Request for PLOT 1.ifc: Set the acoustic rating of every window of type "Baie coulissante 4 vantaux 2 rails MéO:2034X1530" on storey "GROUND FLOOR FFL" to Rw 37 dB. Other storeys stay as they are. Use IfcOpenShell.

First a look at what the model holds.

```python
import ifcopenshell
import ifcopenshell.util.element

model = ifcopenshell.open("PLOT 1.ifc")
print(model.schema)
storey = next(s for s in model.by_type("IfcBuildingStorey") if s.Name == "GROUND FLOOR FFL")
windows = [e for e in ifcopenshell.util.element.get_decomposition(storey) if e.is_a("IfcWindow")]
seen = {}
for e in windows:
    element_type = ifcopenshell.util.element.get_type(e)
    key = (element_type.Name if element_type != e and element_type else None, ifcopenshell.util.element.get_pset(e, "Pset_WindowCommon", "AcousticRating"))
    seen[key] = seen.get(key, 0) + 1
for (name, value), count in sorted(seen.items(), key=str):
    print(count, "x", name, "|", value)
```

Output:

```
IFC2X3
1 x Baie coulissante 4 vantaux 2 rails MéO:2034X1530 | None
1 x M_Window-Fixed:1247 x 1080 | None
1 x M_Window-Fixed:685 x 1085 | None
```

```python
import ifcopenshell
import ifcopenshell.api.pset
import ifcopenshell.util.element

model = ifcopenshell.open("PLOT 1.ifc")

storey = next(s for s in model.by_type("IfcBuildingStorey") if s.Name == "GROUND FLOOR FFL")
windows = [e for e in ifcopenshell.util.element.get_decomposition(storey) if e.is_a("IfcWindow")]

count = 0
for e in windows:
    element_type = ifcopenshell.util.element.get_type(e)
    if element_type in (None, e) or element_type.Name != "Baie coulissante 4 vantaux 2 rails MéO:2034X1530":
        continue
    # add_pset returns the element's existing set when there is one.
    pset = ifcopenshell.api.pset.add_pset(model, product=e, name="Pset_WindowCommon")
    ifcopenshell.api.pset.edit_pset(model, pset=pset, properties={"AcousticRating": "Rw 37 dB"})
    count += 1

print(count, "windows updated")

model.write("PLOT 1-out.ifc")
```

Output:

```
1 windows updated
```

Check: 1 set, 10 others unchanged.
